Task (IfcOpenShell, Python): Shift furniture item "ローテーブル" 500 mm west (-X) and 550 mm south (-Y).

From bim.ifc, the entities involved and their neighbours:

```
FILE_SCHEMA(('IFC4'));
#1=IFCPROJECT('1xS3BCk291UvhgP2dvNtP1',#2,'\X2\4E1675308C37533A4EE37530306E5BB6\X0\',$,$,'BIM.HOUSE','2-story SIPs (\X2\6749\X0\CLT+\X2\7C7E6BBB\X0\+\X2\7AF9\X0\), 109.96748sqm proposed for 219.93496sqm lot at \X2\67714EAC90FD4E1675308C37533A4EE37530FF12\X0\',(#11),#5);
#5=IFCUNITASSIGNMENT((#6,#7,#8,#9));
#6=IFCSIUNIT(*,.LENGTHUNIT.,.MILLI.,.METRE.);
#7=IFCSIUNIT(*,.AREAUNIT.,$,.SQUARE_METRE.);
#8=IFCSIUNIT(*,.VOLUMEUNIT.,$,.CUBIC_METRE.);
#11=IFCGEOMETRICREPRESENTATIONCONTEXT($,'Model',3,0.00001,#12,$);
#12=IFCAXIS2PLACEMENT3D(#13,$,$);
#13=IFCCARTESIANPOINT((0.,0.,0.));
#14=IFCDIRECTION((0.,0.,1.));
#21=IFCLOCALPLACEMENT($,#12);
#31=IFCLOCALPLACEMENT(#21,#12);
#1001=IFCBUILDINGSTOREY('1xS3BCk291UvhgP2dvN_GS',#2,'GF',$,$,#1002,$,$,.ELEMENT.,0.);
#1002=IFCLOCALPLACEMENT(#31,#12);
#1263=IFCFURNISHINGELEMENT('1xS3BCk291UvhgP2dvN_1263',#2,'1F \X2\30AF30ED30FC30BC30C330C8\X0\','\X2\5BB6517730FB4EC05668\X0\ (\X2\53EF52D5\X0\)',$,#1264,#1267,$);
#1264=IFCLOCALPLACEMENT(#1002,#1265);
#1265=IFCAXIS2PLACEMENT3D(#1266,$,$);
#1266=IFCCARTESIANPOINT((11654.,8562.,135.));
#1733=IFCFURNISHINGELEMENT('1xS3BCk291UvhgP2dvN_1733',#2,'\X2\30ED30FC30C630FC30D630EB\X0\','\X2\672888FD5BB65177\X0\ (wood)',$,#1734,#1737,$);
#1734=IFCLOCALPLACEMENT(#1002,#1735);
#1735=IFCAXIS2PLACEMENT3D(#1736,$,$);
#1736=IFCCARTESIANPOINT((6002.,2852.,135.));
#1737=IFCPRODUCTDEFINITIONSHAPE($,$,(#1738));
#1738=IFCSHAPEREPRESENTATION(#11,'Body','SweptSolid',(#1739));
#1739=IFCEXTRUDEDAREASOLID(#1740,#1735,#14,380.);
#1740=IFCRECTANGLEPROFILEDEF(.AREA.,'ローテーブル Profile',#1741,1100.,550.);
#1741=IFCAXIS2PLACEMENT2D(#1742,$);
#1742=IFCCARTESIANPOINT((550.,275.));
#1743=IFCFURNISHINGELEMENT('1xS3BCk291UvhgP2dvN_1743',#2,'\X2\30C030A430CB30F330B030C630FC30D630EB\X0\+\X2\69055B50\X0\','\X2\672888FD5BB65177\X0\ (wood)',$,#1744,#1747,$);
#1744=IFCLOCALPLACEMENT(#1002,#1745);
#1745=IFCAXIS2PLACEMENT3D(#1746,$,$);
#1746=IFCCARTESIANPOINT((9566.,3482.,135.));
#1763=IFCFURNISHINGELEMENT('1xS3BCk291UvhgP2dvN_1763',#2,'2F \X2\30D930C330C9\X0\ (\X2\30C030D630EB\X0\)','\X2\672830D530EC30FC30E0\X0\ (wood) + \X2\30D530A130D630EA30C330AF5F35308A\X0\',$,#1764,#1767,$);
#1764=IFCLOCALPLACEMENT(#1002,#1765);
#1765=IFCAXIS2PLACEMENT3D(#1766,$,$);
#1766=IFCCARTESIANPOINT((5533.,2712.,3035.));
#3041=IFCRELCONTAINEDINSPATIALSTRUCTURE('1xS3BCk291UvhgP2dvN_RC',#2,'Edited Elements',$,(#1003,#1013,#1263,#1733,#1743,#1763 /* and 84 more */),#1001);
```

```python
import ifcopenshell
import ifcopenshell.api.geometry
import ifcopenshell.util.placement

model = ifcopenshell.open("bim.ifc")

item = model.by_guid("1xS3BCk291UvhgP2dvN_1733")
matrix = ifcopenshell.util.placement.get_local_placement(item.ObjectPlacement)
matrix[0, 3] -= 500.0
matrix[1, 3] -= 550.0
ifcopenshell.api.geometry.edit_object_placement(model, product=item, matrix=matrix, is_si=False)

print(ifcopenshell.util.placement.get_local_placement(item.ObjectPlacement).round(3) + 0.0)

model.write("bim-out.ifc")
```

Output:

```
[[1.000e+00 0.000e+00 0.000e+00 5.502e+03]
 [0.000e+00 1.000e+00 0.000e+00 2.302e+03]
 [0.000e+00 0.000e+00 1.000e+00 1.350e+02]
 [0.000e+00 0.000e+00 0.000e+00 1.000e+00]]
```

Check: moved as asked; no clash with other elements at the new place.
